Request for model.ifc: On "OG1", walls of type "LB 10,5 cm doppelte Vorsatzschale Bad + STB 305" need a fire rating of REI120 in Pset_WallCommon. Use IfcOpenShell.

First a look at what the model holds.

```python
import ifcopenshell
import ifcopenshell.util.element

model = ifcopenshell.open("model.ifc")
print(model.schema)
storey = next(s for s in model.by_type("IfcBuildingStorey") if s.Name == "OG1")
walls = [e for e in ifcopenshell.util.element.get_decomposition(storey) if e.is_a("IfcWall")]
seen = {}
for e in walls:
    element_type = ifcopenshell.util.element.get_type(e)
    key = (element_type.Name if element_type != e and element_type else None, ifcopenshell.util.element.get_pset(e, "Pset_WallCommon", "FireRating"))
    seen[key] = seen.get(key, 0) + 1
for (name, value), count in sorted(seen.items(), key=str):
    print(count, "x", name, "|", value)
```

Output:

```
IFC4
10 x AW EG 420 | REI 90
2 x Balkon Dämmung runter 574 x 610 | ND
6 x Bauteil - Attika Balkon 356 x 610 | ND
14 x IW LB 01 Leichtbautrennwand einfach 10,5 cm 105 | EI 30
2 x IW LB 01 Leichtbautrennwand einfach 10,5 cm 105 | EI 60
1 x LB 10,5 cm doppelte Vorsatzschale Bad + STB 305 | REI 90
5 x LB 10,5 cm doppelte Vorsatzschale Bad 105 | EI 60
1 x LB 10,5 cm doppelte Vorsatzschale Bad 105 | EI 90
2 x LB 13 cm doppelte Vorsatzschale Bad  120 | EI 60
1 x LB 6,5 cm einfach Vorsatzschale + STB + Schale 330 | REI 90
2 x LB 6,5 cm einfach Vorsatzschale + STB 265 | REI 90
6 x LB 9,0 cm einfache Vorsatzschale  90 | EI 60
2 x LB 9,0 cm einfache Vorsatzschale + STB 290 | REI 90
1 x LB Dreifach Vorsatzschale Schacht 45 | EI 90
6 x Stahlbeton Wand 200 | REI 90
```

```python
import ifcopenshell
import ifcopenshell.api.pset
import ifcopenshell.util.element

model = ifcopenshell.open("model.ifc")

storey = next(s for s in model.by_type("IfcBuildingStorey") if s.Name == "OG1")
walls = [e for e in ifcopenshell.util.element.get_decomposition(storey) if e.is_a("IfcWall")]

count = 0
for e in walls:
    element_type = ifcopenshell.util.element.get_type(e)
    if element_type in (None, e) or element_type.Name != "LB 10,5 cm doppelte Vorsatzschale Bad + STB 305":
        continue
    # add_pset returns the element's existing set when there is one.
    pset = ifcopenshell.api.pset.add_pset(model, product=e, name="Pset_WallCommon")
    ifcopenshell.api.pset.edit_pset(model, pset=pset, properties={"FireRating": "REI120"})
    count += 1

print(count, "walls updated")

model.write("model_updated.ifc")
```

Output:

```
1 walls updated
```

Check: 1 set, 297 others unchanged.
